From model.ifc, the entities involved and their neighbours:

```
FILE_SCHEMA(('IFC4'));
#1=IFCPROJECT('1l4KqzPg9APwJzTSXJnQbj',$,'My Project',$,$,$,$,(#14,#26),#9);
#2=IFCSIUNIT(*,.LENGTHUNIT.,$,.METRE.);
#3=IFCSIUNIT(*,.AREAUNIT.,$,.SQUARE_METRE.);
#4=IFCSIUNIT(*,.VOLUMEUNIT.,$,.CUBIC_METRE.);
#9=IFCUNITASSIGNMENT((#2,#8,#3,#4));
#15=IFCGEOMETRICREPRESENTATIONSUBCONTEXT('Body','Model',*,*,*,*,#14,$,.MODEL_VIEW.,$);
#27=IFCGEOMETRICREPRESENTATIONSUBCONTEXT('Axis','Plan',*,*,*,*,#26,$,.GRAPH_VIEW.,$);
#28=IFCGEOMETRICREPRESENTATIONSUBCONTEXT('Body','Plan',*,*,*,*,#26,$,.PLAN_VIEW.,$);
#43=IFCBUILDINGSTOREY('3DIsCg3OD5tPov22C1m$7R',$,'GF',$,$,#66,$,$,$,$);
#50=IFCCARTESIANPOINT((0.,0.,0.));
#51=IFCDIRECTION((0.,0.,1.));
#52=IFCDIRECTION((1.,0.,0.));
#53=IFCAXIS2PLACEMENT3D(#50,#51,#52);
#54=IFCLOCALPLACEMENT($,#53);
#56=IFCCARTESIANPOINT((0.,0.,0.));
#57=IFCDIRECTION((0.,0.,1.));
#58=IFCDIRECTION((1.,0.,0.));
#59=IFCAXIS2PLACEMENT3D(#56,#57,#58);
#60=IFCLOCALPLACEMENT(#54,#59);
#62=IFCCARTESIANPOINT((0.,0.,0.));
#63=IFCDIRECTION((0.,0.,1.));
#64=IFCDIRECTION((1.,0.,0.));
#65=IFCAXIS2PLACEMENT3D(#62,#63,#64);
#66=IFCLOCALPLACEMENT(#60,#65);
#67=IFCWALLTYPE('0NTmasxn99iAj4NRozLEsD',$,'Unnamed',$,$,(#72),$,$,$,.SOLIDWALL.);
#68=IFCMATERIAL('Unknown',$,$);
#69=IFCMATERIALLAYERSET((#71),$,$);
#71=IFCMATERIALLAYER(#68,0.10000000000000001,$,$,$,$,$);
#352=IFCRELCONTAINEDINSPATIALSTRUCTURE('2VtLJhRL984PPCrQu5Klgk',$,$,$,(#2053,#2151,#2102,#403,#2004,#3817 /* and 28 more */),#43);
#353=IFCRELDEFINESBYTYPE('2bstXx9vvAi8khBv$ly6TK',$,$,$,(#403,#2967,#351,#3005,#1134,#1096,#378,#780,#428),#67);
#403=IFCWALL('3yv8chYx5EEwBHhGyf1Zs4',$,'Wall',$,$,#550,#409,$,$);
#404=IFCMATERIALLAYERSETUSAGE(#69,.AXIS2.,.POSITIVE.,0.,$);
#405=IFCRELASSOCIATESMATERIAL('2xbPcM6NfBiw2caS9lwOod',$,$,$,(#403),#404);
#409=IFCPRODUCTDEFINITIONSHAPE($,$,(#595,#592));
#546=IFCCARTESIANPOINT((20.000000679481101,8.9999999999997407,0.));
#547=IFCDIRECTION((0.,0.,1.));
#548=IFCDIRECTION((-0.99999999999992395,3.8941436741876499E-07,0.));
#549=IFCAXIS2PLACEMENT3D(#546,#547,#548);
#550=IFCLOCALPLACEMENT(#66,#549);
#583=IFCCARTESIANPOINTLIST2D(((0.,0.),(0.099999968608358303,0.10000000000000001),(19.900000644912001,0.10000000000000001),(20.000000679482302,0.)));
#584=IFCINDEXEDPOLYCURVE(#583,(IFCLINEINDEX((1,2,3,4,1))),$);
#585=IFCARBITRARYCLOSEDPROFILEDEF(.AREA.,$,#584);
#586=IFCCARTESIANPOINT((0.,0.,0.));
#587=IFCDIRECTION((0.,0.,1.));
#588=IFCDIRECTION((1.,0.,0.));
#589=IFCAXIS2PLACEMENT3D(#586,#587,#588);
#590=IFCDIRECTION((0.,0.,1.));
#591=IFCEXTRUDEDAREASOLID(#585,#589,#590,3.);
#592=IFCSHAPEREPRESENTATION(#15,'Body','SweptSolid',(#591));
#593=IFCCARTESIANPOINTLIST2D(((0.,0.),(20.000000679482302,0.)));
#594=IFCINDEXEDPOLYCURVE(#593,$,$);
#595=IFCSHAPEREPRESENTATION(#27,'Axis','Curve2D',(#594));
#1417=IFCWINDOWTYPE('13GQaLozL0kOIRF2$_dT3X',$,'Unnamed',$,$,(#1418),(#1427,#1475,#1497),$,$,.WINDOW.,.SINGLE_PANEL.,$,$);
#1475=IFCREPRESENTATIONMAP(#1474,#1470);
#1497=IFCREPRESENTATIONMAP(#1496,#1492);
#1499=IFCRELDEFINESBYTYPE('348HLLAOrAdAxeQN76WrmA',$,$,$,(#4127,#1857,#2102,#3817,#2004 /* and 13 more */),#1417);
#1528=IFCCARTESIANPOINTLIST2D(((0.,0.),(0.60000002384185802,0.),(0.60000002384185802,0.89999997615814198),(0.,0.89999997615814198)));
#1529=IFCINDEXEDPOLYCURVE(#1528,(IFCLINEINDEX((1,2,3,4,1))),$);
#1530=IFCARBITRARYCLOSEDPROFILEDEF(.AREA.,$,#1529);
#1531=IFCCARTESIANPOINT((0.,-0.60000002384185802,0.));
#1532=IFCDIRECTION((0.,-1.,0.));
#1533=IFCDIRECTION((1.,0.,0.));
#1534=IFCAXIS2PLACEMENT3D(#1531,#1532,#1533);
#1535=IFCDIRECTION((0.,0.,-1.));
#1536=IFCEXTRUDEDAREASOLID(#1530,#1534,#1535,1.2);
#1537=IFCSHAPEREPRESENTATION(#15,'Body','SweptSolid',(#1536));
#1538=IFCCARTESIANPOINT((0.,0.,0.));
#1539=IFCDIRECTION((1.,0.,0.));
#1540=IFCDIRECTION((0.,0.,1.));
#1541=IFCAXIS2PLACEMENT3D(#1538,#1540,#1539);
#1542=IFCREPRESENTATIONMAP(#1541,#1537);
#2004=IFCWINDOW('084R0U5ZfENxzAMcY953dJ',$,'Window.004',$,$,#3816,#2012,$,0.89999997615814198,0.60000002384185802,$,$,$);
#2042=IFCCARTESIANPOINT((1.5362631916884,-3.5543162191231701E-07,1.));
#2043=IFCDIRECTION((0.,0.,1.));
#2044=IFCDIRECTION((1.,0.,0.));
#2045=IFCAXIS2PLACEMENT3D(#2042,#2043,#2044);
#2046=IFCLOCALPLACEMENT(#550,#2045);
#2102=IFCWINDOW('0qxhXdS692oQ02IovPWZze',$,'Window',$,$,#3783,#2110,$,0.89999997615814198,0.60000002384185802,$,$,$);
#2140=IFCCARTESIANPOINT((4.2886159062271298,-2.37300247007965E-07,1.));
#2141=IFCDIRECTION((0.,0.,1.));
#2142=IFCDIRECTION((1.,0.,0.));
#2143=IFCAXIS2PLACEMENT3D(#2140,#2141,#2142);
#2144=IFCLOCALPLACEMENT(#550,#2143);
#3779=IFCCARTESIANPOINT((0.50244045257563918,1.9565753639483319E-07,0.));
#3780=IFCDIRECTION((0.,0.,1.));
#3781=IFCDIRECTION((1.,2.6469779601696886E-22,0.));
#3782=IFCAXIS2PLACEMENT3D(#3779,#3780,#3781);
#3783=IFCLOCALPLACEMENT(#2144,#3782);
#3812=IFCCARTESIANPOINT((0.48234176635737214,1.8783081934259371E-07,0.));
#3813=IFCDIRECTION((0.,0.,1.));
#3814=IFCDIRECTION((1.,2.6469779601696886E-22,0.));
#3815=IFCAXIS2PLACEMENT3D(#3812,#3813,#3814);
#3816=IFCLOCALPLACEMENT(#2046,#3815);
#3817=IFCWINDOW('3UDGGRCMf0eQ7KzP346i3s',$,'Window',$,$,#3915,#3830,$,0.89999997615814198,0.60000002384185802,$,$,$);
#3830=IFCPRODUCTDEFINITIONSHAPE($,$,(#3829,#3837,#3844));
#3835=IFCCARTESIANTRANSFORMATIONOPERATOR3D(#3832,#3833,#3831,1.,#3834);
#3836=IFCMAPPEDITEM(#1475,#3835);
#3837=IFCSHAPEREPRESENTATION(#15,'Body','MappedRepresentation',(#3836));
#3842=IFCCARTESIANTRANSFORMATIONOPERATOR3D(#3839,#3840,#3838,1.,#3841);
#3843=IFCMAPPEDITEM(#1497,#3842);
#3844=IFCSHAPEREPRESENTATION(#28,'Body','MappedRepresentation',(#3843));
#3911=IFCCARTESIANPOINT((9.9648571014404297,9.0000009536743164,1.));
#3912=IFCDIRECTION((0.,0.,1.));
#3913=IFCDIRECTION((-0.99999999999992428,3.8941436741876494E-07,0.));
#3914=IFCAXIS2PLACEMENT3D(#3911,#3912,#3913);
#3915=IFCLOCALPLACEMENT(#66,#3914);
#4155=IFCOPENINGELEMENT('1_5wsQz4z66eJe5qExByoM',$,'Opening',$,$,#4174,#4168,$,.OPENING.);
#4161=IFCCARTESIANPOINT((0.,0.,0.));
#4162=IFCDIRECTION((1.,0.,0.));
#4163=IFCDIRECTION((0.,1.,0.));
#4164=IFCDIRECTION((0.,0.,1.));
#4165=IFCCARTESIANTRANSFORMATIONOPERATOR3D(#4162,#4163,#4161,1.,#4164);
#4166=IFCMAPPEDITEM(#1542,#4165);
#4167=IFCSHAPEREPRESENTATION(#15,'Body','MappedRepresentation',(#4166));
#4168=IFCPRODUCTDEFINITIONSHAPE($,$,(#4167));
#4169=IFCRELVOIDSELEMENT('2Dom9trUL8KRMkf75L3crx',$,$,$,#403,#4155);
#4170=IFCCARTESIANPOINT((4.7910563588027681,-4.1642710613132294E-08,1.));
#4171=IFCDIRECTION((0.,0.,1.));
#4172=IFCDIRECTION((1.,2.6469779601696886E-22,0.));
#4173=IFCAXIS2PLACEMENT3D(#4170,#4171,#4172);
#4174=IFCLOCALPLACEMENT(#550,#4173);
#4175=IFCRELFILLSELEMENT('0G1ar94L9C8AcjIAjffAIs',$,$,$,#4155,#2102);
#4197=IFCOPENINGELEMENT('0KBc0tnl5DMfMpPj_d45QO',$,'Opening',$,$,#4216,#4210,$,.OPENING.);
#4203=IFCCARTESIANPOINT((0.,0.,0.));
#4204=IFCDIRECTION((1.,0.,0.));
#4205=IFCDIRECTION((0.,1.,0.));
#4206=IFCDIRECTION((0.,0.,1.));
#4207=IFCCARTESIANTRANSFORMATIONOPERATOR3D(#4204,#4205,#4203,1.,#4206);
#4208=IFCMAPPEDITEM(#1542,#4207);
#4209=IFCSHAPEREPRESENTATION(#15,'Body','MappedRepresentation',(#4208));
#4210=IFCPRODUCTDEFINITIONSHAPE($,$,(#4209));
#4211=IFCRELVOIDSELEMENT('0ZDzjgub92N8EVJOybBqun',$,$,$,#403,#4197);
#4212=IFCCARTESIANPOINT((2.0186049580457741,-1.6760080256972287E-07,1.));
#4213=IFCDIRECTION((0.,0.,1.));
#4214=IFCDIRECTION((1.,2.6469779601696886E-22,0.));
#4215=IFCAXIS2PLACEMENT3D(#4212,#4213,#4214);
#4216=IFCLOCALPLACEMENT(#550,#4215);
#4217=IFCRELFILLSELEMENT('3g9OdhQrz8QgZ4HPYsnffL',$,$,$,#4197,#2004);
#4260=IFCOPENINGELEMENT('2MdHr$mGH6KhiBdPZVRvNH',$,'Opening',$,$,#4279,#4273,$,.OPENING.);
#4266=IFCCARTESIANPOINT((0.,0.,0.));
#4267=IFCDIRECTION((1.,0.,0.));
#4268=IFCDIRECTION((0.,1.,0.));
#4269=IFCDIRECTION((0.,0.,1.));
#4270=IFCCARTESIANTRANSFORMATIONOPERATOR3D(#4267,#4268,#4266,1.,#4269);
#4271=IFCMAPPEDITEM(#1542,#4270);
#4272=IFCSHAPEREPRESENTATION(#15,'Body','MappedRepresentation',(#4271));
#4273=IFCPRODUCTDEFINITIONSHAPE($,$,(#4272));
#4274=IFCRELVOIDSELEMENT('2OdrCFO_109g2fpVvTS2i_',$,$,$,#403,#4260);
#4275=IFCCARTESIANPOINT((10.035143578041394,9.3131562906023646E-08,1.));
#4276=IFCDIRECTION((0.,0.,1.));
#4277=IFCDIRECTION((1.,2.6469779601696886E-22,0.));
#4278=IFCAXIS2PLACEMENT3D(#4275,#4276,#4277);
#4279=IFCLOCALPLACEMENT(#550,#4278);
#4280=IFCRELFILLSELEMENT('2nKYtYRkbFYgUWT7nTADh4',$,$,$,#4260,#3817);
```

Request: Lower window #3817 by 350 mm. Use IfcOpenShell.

```python
import numpy as np
import ifcopenshell
import ifcopenshell.api.geometry
import ifcopenshell.util.placement
import ifcopenshell.util.unit

model = ifcopenshell.open("model.ifc")
unit_scale = ifcopenshell.util.unit.calculate_unit_scale(model)

window = model.by_guid("3UDGGRCMf0eQ7KzP346i3s")
opening = window.FillsVoids[0].RelatingOpeningElement
dz = -0.35

shift = np.array([0.0, 0.0, dz])
# The window is not placed relative to its opening, so move both.
for product in (opening, window):
    matrix = ifcopenshell.util.placement.get_local_placement(product.ObjectPlacement)
    matrix[:3, 3] += shift
    ifcopenshell.api.geometry.edit_object_placement(model, product=product, matrix=matrix, is_si=False)

print(f"moved by {dz * unit_scale:+.3f} m")

model.write("model_edited.ifc")
```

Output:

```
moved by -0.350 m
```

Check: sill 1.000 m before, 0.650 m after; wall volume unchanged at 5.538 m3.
